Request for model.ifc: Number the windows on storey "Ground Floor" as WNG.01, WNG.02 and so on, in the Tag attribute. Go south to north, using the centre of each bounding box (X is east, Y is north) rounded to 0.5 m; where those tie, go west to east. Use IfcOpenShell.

First a look at what the model holds.

```python
import ifcopenshell
import ifcopenshell.util.element
import ifcopenshell.util.placement

model = ifcopenshell.open("model.ifc")
print(model.schema)
storey = next(s for s in model.by_type("IfcBuildingStorey") if s.Name == "Ground Floor")
windows = [e for e in ifcopenshell.util.element.get_decomposition(storey) if e.is_a("IfcWindow")]
for e in sorted(windows, key=lambda e: e.id()):
    origin = ifcopenshell.util.placement.get_local_placement(e.ObjectPlacement)[:3, 3]
    print(e.id(), e.Tag, e.Name, origin.round(2) + 0.0, sep=" | ")
```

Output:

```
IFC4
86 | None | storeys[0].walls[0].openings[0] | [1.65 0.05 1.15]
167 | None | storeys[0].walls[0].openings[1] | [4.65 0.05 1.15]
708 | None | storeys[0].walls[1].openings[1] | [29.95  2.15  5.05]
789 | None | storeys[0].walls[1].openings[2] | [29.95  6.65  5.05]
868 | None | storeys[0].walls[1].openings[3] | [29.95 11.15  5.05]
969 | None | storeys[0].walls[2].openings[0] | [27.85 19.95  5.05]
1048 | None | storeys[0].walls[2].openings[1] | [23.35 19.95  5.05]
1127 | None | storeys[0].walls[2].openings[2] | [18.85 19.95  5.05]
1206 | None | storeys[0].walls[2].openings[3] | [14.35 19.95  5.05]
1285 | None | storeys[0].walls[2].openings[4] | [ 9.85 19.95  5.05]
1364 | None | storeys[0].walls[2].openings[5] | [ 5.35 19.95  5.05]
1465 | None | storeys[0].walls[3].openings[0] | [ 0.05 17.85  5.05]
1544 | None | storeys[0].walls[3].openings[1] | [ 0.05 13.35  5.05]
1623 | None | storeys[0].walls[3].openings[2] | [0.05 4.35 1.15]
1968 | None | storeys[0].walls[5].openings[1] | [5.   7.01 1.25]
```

```python
import ifcopenshell
import ifcopenshell.geom
import ifcopenshell.util.element
import ifcopenshell.util.shape

model = ifcopenshell.open("model.ifc")
settings = ifcopenshell.geom.settings()
settings.set("use-world-coords", True)


def centre(element):
    shape = ifcopenshell.geom.create_shape(settings, element)
    return ifcopenshell.util.shape.get_bbox_centroid(shape.geometry)


storey = next(s for s in model.by_type("IfcBuildingStorey") if s.Name == "Ground Floor")
windows = [e for e in ifcopenshell.util.element.get_decomposition(storey) if e.is_a("IfcWindow")]

# Insertion points can sit at a corner or the storey origin, so sort by the geometry (in metres).
centres = {e: centre(e) for e in windows}
windows.sort(key=lambda e: (round(centres[e][1] / 0.5), centres[e][0]))

for i, e in enumerate(windows, start=1):
    number = f"WNG.{i:02d}"
    e.Tag = number
    print(e.id(), number)

model.write("model_v2.ifc")
```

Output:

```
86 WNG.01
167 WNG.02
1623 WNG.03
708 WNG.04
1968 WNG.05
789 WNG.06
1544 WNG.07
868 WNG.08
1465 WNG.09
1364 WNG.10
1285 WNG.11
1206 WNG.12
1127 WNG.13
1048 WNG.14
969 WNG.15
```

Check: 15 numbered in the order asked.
